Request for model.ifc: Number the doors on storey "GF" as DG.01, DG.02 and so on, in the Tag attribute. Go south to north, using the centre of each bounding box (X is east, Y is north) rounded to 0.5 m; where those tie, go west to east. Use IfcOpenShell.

First a look at what the model holds.

```python
import ifcopenshell
import ifcopenshell.util.element
import ifcopenshell.util.placement

model = ifcopenshell.open("model.ifc")
print(model.schema)
storey = next(s for s in model.by_type("IfcBuildingStorey") if s.Name == "GF")
doors = [e for e in ifcopenshell.util.element.get_decomposition(storey) if e.is_a("IfcDoor")]
for e in sorted(doors, key=lambda e: e.id()):
    origin = ifcopenshell.util.placement.get_local_placement(e.ObjectPlacement)[:3, 3]
    print(e.id(), e.Tag, e.Name, origin.round(2) + 0.0, sep=" | ")
```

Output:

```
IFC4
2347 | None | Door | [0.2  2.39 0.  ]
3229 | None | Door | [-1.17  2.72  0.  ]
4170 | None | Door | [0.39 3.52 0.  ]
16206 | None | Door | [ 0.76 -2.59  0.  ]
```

```python
import ifcopenshell
import ifcopenshell.geom
import ifcopenshell.util.element
import ifcopenshell.util.shape

model = ifcopenshell.open("model.ifc")
settings = ifcopenshell.geom.settings()
settings.set("use-world-coords", True)


def centre(element):
    shape = ifcopenshell.geom.create_shape(settings, element)
    return ifcopenshell.util.shape.get_bbox_centroid(shape.geometry)


storey = next(s for s in model.by_type("IfcBuildingStorey") if s.Name == "GF")
doors = [e for e in ifcopenshell.util.element.get_decomposition(storey) if e.is_a("IfcDoor")]

# Insertion points can sit at a corner or the storey origin, so sort by the geometry (in metres).
centres = {e: centre(e) for e in doors}
doors.sort(key=lambda e: (round(centres[e][1] / 0.5), centres[e][0]))

for i, e in enumerate(doors, start=1):
    number = f"DG.{i:02d}"
    e.Tag = number
    print(e.id(), number)

model.write("model_v2.ifc")
```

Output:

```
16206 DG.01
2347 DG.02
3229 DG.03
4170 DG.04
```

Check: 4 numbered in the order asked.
